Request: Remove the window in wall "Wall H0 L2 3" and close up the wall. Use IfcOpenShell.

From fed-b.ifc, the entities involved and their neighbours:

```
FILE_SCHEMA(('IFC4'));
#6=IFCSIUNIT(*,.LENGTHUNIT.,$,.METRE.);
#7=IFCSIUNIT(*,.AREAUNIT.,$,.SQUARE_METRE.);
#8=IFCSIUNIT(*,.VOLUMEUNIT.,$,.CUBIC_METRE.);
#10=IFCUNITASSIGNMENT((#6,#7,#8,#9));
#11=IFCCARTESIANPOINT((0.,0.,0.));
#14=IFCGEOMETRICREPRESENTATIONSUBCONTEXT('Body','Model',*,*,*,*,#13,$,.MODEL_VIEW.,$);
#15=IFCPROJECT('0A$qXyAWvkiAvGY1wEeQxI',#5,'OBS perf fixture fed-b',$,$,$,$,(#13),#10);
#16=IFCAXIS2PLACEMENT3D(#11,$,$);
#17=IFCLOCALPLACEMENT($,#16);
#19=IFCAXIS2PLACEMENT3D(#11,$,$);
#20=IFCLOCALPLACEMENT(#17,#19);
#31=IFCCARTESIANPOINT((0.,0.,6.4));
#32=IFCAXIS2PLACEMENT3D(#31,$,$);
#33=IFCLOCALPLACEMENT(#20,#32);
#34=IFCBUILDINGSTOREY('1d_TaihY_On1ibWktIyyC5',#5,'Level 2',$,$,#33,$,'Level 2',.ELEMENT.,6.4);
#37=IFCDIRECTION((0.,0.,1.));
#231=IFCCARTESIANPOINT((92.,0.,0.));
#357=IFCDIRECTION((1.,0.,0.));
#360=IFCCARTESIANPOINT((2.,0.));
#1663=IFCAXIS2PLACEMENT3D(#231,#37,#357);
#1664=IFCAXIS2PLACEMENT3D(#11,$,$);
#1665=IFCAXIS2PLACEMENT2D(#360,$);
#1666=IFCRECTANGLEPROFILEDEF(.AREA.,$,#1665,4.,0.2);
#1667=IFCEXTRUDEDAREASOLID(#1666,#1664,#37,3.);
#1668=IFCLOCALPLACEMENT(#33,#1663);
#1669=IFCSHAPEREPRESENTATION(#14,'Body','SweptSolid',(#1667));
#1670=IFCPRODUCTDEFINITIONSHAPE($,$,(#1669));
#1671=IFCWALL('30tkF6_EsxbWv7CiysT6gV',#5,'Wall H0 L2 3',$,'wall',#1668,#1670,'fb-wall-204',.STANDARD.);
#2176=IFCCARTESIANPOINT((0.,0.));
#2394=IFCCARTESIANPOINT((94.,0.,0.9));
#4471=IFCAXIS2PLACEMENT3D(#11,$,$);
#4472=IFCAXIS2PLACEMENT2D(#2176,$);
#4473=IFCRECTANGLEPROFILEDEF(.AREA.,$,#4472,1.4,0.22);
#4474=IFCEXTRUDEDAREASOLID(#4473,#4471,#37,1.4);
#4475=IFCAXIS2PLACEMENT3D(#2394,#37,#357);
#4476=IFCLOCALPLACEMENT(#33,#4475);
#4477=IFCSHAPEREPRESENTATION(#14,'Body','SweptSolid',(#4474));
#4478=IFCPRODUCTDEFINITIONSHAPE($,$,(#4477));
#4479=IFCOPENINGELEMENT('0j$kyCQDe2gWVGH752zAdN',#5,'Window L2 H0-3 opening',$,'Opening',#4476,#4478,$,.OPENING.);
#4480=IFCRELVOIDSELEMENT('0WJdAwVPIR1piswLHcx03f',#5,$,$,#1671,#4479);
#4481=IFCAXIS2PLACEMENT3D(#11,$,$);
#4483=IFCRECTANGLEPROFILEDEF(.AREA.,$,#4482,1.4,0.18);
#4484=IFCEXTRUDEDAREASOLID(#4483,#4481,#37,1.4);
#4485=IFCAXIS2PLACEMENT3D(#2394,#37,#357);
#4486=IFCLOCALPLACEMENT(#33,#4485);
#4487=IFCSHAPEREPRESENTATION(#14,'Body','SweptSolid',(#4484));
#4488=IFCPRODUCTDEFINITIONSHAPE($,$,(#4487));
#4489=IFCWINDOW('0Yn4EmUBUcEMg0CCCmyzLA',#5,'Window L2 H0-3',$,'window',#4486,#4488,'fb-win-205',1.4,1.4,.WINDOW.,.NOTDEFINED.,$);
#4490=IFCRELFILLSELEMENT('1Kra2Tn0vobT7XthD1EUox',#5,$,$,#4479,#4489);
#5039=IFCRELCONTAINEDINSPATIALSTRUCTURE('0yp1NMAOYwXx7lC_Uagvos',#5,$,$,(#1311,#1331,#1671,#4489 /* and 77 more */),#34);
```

```python
import ifcopenshell
import ifcopenshell.api.feature
import ifcopenshell.api.root
import ifcopenshell.geom
import ifcopenshell.util.shape

model = ifcopenshell.open("fed-b.ifc")
settings = ifcopenshell.geom.settings()


def volume(element):
    """Net volume in cubic metres, openings subtracted."""
    shape = ifcopenshell.geom.create_shape(settings, element)
    return ifcopenshell.util.shape.get_volume(shape.geometry)


window = model.by_id(4489)
opening = window.FillsVoids[0].RelatingOpeningElement
wall = opening.VoidsElements[0].RelatingBuildingElement
before = volume(wall)

ifcopenshell.api.root.remove_product(model, product=window)
ifcopenshell.api.feature.remove_feature(model, feature=opening)

after = volume(wall)

print(f"wall volume {before:.3f} -> {after:.3f} m3")

model.write("fed-b_v2.ifc")
```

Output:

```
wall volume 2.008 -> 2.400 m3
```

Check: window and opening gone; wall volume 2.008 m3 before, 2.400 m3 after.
